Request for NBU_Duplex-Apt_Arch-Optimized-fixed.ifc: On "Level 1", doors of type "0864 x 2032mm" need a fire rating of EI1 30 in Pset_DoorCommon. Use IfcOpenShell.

First a look at what the model holds.

```python
import ifcopenshell
import ifcopenshell.util.element

model = ifcopenshell.open("NBU_Duplex-Apt_Arch-Optimized-fixed.ifc")
print(model.schema)
storey = next(s for s in model.by_type("IfcBuildingStorey") if s.Name == "Level 1")
doors = [e for e in ifcopenshell.util.element.get_decomposition(storey) if e.is_a("IfcDoor")]
seen = {}
for e in doors:
    element_type = ifcopenshell.util.element.get_type(e)
    key = (element_type.Name if element_type != e and element_type else None, ifcopenshell.util.element.get_pset(e, "Pset_DoorCommon", "FireRating"))
    seen[key] = seen.get(key, 0) + 1
for (name, value), count in sorted(seen.items(), key=str):
    print(count, "x", name, "|", value)
```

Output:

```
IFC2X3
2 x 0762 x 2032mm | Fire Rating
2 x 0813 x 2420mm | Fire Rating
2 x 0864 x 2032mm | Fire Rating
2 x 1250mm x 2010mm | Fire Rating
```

```python
import ifcopenshell
import ifcopenshell.api.pset
import ifcopenshell.util.element

model = ifcopenshell.open("NBU_Duplex-Apt_Arch-Optimized-fixed.ifc")

storey = next(s for s in model.by_type("IfcBuildingStorey") if s.Name == "Level 1")
doors = [e for e in ifcopenshell.util.element.get_decomposition(storey) if e.is_a("IfcDoor")]

count = 0
for e in doors:
    element_type = ifcopenshell.util.element.get_type(e)
    if element_type in (None, e) or element_type.Name != "0864 x 2032mm":
        continue
    # add_pset returns the element's existing set when there is one.
    pset = ifcopenshell.api.pset.add_pset(model, product=e, name="Pset_DoorCommon")
    ifcopenshell.api.pset.edit_pset(model, pset=pset, properties={"FireRating": "EI1 30"})
    count += 1

print(count, "doors updated")

model.write("NBU_Duplex-Apt_Arch-Optimized-fixed_rev.ifc")
```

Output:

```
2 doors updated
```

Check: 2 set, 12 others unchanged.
